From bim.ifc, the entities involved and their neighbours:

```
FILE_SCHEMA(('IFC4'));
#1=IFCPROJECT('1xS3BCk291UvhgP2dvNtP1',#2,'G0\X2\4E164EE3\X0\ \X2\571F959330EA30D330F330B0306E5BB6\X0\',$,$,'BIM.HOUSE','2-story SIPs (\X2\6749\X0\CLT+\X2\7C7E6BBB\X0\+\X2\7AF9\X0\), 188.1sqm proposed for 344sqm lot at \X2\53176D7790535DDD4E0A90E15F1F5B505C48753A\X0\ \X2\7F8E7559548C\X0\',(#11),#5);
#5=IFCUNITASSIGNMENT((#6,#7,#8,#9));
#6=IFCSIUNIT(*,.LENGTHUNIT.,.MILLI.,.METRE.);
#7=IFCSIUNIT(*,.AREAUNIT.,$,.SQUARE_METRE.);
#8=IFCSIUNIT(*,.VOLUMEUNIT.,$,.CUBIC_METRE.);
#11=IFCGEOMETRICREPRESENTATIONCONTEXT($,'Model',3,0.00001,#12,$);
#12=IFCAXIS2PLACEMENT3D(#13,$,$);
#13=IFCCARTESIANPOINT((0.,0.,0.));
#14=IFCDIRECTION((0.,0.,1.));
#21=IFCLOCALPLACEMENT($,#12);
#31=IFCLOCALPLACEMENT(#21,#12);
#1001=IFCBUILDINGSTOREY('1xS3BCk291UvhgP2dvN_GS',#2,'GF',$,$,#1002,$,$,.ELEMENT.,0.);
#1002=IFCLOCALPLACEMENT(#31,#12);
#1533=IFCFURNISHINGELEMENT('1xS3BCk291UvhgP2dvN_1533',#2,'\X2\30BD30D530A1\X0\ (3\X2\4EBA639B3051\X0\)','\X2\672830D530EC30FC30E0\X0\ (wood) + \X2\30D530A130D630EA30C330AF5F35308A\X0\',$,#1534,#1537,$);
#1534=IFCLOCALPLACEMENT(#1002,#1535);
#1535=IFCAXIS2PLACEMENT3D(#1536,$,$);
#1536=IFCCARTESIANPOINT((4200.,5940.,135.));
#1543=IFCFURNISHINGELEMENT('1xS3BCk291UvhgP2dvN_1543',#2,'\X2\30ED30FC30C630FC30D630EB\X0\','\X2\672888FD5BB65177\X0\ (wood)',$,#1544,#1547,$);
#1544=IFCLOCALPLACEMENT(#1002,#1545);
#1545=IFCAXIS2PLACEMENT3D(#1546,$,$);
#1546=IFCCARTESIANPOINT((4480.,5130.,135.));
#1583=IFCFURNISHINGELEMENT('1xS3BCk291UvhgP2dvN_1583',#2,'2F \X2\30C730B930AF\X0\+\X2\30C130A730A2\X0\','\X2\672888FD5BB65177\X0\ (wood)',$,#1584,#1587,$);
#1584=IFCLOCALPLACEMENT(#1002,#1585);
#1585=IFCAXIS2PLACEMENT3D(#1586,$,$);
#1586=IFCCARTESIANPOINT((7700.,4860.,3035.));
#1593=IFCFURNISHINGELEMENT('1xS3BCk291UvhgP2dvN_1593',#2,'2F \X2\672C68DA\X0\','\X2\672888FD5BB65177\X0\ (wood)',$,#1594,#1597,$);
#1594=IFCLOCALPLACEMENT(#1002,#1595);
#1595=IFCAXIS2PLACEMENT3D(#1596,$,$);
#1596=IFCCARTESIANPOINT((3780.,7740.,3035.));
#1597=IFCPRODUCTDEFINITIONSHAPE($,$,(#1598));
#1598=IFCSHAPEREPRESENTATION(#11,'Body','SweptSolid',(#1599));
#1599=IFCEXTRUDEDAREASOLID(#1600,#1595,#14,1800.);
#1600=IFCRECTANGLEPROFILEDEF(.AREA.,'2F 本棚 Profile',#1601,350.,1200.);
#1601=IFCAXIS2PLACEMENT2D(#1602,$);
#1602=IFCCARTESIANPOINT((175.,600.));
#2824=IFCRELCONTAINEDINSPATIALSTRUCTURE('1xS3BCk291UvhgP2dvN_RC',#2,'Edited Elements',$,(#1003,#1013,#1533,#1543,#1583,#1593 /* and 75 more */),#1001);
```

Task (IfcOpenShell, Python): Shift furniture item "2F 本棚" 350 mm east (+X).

```python
import ifcopenshell
import ifcopenshell.api.geometry
import ifcopenshell.util.placement

model = ifcopenshell.open("bim.ifc")

item = model.by_guid("1xS3BCk291UvhgP2dvN_1593")
matrix = ifcopenshell.util.placement.get_local_placement(item.ObjectPlacement)
matrix[0, 3] += 350.0
ifcopenshell.api.geometry.edit_object_placement(model, product=item, matrix=matrix, is_si=False)

print(ifcopenshell.util.placement.get_local_placement(item.ObjectPlacement).round(3) + 0.0)

model.write("bim_updated.ifc")
```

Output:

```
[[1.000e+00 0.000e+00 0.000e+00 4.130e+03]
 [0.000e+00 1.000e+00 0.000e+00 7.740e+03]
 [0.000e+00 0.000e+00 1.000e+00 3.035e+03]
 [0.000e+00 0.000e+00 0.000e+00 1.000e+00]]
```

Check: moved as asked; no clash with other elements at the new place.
